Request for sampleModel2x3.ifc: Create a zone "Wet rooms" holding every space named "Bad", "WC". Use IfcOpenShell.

First a look at what the model holds.

```python
import ifcopenshell

model = ifcopenshell.open("sampleModel2x3.ifc")
print(model.schema)
seen = {}
for space in model.by_type("IfcSpace"):
    seen[space.LongName] = seen.get(space.LongName, 0) + 1
for name, count in sorted(seen.items(), key=str):
    print(count, "x", name)
print("zones:", [z.Name for z in model.by_type("IfcZone")][:20])
```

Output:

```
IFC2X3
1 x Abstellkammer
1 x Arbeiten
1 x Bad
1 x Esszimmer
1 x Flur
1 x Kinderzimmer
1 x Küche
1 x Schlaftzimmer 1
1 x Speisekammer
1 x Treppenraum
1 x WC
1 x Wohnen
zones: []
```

```python
import ifcopenshell
import ifcopenshell.api.group
import ifcopenshell.api.root

model = ifcopenshell.open("sampleModel2x3.ifc")

names = {"Bad", "WC"}
spaces = [s for s in model.by_type("IfcSpace") if s.LongName in names]

zone = ifcopenshell.api.root.create_entity(model, ifc_class="IfcZone", name="Wet rooms")
ifcopenshell.api.group.assign_group(model, products=spaces, group=zone)
print(len(spaces), "spaces in", zone.Name)

model.write("sampleModel2x3_rev.ifc")
```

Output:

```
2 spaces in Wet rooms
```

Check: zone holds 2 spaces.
